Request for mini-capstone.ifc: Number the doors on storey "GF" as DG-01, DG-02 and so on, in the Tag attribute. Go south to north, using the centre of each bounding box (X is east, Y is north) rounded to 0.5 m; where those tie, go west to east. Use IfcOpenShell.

First a look at what the model holds.

```python
import ifcopenshell
import ifcopenshell.util.element
import ifcopenshell.util.placement

model = ifcopenshell.open("mini-capstone.ifc")
print(model.schema)
storey = next(s for s in model.by_type("IfcBuildingStorey") if s.Name == "GF")
doors = [e for e in ifcopenshell.util.element.get_decomposition(storey) if e.is_a("IfcDoor")]
for e in sorted(doors, key=lambda e: e.id()):
    origin = ifcopenshell.util.placement.get_local_placement(e.ObjectPlacement)[:3, 3]
    print(e.id(), e.Tag, e.Name, origin.round(2) + 0.0, sep=" | ")
```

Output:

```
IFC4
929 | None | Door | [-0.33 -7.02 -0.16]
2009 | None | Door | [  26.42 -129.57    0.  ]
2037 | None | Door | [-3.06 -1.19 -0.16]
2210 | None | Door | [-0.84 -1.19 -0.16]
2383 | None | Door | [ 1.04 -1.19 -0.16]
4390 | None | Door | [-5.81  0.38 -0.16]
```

```python
import ifcopenshell
import ifcopenshell.geom
import ifcopenshell.util.element
import ifcopenshell.util.shape

model = ifcopenshell.open("mini-capstone.ifc")
settings = ifcopenshell.geom.settings()
settings.set("use-world-coords", True)


def centre(element):
    shape = ifcopenshell.geom.create_shape(settings, element)
    return ifcopenshell.util.shape.get_bbox_centroid(shape.geometry)


storey = next(s for s in model.by_type("IfcBuildingStorey") if s.Name == "GF")
doors = [e for e in ifcopenshell.util.element.get_decomposition(storey) if e.is_a("IfcDoor")]

# Insertion points can sit at a corner or the storey origin, so sort by the geometry (in metres).
centres = {e: centre(e) for e in doors}
doors.sort(key=lambda e: (round(centres[e][1] / 0.5), centres[e][0]))

for i, e in enumerate(doors, start=1):
    number = f"DG-{i:02d}"
    e.Tag = number
    print(e.id(), number)

model.write("mini-capstone_v2.ifc")
```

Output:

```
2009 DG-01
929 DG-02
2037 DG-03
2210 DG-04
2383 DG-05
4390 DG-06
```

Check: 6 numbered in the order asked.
